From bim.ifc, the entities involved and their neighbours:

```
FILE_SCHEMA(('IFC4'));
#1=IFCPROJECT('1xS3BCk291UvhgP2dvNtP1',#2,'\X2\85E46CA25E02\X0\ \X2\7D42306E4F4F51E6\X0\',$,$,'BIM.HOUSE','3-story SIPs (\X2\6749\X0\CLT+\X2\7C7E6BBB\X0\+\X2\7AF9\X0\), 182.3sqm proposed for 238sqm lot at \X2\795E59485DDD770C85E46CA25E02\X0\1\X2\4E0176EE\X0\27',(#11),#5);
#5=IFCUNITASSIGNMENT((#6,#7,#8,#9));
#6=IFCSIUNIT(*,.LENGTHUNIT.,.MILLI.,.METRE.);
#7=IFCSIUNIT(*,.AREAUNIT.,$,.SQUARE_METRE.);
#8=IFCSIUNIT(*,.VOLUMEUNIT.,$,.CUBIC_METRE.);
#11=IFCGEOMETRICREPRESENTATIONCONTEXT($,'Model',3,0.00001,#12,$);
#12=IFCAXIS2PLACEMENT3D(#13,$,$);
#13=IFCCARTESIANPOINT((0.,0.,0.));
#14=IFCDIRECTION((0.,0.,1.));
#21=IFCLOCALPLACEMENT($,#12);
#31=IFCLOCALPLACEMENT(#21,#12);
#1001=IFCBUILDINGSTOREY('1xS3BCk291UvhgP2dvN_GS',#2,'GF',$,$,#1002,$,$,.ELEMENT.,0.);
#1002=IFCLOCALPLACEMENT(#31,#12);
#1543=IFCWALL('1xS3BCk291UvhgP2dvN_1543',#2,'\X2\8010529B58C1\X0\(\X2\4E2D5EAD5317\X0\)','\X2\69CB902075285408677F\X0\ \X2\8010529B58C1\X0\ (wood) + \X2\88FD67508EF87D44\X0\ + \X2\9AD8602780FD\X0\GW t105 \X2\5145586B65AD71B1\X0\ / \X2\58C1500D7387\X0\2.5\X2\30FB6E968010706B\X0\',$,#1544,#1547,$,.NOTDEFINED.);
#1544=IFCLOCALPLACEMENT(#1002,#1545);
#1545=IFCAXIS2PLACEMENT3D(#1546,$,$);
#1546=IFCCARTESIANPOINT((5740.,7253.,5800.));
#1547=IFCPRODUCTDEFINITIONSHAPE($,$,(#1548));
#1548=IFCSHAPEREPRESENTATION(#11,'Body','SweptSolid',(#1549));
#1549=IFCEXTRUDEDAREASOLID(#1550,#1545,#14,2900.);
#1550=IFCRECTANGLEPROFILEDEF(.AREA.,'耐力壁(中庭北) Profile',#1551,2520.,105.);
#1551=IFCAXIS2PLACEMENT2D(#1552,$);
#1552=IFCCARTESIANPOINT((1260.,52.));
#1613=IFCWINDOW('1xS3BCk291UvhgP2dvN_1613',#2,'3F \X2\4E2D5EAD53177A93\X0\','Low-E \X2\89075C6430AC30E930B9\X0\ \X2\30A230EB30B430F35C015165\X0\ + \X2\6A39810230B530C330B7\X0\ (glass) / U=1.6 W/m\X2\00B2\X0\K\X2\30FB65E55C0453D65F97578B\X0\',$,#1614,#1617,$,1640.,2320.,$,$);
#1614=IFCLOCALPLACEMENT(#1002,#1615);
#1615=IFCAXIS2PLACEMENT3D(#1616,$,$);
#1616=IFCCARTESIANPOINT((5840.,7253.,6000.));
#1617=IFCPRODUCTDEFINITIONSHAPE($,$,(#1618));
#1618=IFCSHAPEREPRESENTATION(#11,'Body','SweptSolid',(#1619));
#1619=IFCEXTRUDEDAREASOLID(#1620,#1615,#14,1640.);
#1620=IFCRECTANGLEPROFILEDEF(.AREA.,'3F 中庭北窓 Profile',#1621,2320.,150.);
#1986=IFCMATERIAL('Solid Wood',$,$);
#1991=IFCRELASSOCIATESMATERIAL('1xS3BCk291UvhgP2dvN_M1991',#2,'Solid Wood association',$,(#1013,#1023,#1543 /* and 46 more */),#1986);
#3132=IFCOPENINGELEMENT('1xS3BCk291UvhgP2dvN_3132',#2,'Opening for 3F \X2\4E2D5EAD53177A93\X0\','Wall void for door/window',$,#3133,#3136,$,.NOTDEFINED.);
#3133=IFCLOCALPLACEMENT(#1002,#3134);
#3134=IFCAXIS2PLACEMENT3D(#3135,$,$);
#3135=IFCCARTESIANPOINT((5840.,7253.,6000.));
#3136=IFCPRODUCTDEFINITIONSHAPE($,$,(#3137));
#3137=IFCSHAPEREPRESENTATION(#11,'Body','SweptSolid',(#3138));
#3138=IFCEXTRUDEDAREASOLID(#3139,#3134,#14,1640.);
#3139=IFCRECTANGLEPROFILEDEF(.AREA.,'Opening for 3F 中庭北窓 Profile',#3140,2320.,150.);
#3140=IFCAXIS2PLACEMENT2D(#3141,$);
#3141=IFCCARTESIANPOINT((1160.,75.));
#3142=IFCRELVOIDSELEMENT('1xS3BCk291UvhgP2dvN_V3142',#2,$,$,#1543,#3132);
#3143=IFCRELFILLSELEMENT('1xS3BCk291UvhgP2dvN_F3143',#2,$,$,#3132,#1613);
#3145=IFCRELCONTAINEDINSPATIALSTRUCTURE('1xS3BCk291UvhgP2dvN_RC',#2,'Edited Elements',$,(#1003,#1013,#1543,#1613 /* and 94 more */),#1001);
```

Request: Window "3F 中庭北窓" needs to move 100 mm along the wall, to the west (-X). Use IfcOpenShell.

```python
import ifcopenshell
import ifcopenshell.api.geometry
import ifcopenshell.util.placement
import ifcopenshell.util.unit

model = ifcopenshell.open("bim.ifc")
unit_scale = ifcopenshell.util.unit.calculate_unit_scale(model)

window = model.by_guid("1xS3BCk291UvhgP2dvN_1613")
opening = window.FillsVoids[0].RelatingOpeningElement
wall = opening.VoidsElements[0].RelatingBuildingElement

wall_matrix = ifcopenshell.util.placement.get_local_placement(wall.ObjectPlacement)
shift = wall_matrix[:3, 0] * -0.1 / unit_scale
before = ifcopenshell.util.placement.get_local_placement(window.ObjectPlacement)[:3, 3].copy()

# The window is not placed relative to its opening, so move both.
for product in (opening, window):
    matrix = ifcopenshell.util.placement.get_local_placement(product.ObjectPlacement)
    matrix[:3, 3] += shift
    ifcopenshell.api.geometry.edit_object_placement(model, product=product, matrix=matrix, is_si=False)

after = ifcopenshell.util.placement.get_local_placement(window.ObjectPlacement)[:3, 3]
print("window moved by", (after - before).round(3) + 0.0)

model.write("bim_v2.ifc")
```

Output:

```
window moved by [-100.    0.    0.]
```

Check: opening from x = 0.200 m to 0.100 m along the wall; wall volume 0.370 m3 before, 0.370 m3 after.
